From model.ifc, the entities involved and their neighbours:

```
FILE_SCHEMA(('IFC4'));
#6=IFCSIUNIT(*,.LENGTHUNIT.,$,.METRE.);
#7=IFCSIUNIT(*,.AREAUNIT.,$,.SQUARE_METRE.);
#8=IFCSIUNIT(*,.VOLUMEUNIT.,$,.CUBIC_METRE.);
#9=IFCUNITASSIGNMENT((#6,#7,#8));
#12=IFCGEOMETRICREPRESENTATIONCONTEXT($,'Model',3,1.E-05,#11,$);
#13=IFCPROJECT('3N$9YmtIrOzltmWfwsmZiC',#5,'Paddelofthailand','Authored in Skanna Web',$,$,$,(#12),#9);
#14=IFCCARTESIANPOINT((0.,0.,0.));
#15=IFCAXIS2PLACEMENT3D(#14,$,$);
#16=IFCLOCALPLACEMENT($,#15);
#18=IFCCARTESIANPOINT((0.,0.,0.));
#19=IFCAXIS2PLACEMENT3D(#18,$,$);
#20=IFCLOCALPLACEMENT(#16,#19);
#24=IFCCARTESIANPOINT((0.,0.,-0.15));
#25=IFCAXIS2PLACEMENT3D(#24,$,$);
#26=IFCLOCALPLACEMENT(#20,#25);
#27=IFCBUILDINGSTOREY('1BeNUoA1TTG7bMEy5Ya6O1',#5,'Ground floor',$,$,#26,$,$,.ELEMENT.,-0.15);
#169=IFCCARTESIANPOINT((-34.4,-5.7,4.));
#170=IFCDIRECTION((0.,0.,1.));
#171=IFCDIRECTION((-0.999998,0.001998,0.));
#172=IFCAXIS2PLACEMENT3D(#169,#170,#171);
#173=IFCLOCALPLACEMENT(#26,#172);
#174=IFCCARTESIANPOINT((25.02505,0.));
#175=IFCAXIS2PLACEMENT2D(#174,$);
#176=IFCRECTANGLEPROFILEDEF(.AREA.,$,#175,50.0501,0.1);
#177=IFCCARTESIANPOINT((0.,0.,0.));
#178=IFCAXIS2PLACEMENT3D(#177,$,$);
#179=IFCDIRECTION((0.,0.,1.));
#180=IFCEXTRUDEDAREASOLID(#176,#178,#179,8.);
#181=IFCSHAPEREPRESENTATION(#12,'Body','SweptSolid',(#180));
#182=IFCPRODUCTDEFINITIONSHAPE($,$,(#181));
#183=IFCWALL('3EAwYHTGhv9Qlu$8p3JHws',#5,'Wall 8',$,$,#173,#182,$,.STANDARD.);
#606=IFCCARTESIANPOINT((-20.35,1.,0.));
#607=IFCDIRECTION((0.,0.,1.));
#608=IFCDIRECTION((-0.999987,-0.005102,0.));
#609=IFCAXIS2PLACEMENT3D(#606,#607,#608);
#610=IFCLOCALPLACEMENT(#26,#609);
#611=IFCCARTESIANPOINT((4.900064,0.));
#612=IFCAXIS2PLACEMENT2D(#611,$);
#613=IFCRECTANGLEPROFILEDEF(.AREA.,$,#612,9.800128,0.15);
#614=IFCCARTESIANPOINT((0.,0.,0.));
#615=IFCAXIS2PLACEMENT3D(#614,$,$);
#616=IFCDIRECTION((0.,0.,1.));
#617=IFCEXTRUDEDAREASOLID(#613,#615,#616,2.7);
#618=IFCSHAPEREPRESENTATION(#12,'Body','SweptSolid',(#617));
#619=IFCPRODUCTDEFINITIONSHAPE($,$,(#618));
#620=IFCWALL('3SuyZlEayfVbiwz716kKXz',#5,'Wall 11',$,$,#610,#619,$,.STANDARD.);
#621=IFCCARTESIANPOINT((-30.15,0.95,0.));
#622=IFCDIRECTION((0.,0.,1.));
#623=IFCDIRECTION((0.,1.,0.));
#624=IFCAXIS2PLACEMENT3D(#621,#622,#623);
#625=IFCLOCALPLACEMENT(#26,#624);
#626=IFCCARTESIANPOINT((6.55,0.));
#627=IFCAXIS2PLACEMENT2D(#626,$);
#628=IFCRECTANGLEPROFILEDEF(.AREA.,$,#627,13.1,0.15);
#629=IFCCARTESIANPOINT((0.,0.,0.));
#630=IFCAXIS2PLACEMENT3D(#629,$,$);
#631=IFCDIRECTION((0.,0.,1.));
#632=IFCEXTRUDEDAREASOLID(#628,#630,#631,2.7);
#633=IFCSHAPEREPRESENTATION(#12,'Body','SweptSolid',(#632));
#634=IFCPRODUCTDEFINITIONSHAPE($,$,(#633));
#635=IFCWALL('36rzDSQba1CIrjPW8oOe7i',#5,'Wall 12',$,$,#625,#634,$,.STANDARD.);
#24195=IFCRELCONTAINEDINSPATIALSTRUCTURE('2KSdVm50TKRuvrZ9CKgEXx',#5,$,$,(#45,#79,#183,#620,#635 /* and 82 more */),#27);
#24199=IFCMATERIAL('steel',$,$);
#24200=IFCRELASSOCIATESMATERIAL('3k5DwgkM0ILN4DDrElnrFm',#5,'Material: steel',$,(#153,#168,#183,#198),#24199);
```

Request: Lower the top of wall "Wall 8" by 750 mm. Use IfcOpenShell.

```python
import ifcopenshell
import ifcopenshell.geom
import ifcopenshell.util.shape
import ifcopenshell.util.unit

model = ifcopenshell.open("model.ifc")
unit_scale = ifcopenshell.util.unit.calculate_unit_scale(model)
settings = ifcopenshell.geom.settings()


def volume(element):
    """Net volume in cubic metres, openings subtracted."""
    shape = ifcopenshell.geom.create_shape(settings, element)
    return ifcopenshell.util.shape.get_volume(shape.geometry)


wall = model.by_guid("3EAwYHTGhv9Qlu$8p3JHws")
before = volume(wall)

body = next(r for r in wall.Representation.Representations if r.RepresentationIdentifier == "Body")
solid = body.Items[0]
old_height = solid.Depth
solid.Depth -= 0.75 / unit_scale
after = volume(wall)

print(f"height {old_height:g} -> {solid.Depth:g}, volume {before:.3f} -> {after:.3f} m3")

model.write("model_updated.ifc")
```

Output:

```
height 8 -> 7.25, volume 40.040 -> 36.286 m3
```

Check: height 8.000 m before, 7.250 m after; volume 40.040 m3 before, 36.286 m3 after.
